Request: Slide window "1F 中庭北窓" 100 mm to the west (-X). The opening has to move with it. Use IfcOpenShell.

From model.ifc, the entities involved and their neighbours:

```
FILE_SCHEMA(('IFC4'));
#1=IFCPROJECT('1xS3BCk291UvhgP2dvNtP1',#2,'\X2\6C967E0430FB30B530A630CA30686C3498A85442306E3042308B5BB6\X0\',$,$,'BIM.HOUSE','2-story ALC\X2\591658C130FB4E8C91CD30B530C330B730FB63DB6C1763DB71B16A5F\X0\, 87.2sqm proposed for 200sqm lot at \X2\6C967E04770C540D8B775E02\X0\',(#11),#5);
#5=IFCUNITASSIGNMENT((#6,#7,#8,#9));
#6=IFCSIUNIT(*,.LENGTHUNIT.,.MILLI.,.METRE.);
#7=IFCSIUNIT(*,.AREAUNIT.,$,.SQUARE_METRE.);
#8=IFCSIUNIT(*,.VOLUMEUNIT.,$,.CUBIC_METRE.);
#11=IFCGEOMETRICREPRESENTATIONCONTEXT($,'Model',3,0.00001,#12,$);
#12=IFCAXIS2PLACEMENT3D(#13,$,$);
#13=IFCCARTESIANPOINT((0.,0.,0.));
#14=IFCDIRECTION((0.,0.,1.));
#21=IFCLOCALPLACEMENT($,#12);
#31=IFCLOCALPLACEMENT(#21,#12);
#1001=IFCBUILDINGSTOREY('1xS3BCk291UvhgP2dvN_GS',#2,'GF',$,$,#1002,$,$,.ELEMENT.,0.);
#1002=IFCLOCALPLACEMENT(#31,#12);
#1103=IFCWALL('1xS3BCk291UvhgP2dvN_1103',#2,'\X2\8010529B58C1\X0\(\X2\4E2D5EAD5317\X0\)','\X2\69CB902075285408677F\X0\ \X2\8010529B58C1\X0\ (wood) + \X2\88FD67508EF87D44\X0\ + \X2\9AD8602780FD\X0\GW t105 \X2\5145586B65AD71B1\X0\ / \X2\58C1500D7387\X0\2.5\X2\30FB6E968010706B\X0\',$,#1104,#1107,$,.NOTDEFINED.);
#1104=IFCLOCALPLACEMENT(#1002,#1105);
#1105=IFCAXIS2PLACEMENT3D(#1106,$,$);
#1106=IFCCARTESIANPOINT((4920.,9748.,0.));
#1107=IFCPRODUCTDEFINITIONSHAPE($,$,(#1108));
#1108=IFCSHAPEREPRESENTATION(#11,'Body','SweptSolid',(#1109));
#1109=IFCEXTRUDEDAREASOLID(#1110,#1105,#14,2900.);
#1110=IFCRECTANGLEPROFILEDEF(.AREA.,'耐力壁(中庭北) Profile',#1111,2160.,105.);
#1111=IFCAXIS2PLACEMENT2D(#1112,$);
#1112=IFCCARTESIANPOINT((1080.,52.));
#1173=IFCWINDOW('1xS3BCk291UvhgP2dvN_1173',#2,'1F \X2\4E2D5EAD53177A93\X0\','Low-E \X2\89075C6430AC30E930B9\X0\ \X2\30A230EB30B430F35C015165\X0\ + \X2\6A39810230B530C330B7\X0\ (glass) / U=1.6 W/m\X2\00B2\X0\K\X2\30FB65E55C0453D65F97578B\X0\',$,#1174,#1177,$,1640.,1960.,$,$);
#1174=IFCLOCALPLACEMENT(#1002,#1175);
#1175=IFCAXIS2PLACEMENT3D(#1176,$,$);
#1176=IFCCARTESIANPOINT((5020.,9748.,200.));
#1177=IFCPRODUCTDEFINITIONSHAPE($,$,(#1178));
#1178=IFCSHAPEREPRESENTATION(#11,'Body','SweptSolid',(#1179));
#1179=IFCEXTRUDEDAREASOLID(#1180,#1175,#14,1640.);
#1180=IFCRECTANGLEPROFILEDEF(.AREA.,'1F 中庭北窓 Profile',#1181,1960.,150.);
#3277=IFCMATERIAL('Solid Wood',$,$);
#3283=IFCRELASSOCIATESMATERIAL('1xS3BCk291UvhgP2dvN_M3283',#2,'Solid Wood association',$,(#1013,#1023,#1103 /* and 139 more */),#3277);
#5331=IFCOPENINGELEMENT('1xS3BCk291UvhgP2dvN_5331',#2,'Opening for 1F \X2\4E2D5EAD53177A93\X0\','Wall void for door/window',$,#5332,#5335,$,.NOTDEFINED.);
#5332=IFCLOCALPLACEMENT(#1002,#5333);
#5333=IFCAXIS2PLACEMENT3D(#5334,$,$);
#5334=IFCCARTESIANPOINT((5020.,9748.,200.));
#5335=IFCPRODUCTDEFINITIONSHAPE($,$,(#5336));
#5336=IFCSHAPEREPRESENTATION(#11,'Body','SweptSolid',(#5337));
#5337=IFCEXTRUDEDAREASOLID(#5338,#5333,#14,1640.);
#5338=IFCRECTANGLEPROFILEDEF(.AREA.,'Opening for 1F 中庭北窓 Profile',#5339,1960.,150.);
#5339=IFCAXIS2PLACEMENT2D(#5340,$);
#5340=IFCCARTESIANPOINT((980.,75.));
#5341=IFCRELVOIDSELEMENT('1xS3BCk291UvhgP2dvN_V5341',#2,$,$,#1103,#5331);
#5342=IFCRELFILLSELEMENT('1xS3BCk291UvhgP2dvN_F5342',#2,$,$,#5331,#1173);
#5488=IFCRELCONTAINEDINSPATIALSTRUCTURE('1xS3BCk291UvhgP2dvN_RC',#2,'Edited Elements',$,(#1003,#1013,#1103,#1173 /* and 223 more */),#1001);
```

```python
import ifcopenshell
import ifcopenshell.api.geometry
import ifcopenshell.util.placement
import ifcopenshell.util.unit

model = ifcopenshell.open("model.ifc")
unit_scale = ifcopenshell.util.unit.calculate_unit_scale(model)

window = model.by_id(1173)
opening = window.FillsVoids[0].RelatingOpeningElement
wall = opening.VoidsElements[0].RelatingBuildingElement

wall_matrix = ifcopenshell.util.placement.get_local_placement(wall.ObjectPlacement)
shift = wall_matrix[:3, 0] * -0.1 / unit_scale
before = ifcopenshell.util.placement.get_local_placement(window.ObjectPlacement)[:3, 3].copy()

# The window is not placed relative to its opening, so move both.
for product in (opening, window):
    matrix = ifcopenshell.util.placement.get_local_placement(product.ObjectPlacement)
    matrix[:3, 3] += shift
    ifcopenshell.api.geometry.edit_object_placement(model, product=product, matrix=matrix, is_si=False)

after = ifcopenshell.util.placement.get_local_placement(window.ObjectPlacement)[:3, 3]
print("window moved by", (after - before).round(3) + 0.0)

model.write("model_rev.ifc")
```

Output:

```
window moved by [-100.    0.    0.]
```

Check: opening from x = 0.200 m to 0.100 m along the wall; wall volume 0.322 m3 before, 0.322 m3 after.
